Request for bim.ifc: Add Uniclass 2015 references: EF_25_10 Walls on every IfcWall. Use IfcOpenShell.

First a look at what the model holds.

```python
import ifcopenshell

model = ifcopenshell.open("bim.ifc")
print(model.schema)
print("classifications:", [c.Name for c in model.by_type("IfcClassification")])
for ifc_class in ("IfcDoor", "IfcRoof", "IfcStair", "IfcWall", "IfcWindow"):
    print(ifc_class, len(model.by_type(ifc_class)))
```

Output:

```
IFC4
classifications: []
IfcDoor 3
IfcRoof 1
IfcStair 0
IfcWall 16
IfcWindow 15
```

```python
import ifcopenshell
import ifcopenshell.api.classification

model = ifcopenshell.open("bim.ifc")

system = ifcopenshell.api.classification.add_classification(model, classification="Uniclass 2015")

codes = {
    "IfcWall": ("EF_25_10", "Walls"),
}
for ifc_class, (code, name) in codes.items():
    products = model.by_type(ifc_class)
    ifcopenshell.api.classification.add_reference(
        model, products=products, classification=system, identification=code, name=name
    )
    print(code, len(products))

model.write("bim_v2.ifc")
```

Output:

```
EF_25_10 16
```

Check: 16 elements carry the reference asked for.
